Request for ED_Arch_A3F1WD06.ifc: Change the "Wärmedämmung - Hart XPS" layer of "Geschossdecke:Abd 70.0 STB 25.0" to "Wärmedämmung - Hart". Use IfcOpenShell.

First a look at what the model holds.

```python
import ifcopenshell
import ifcopenshell.util.element

model = ifcopenshell.open("ED_Arch_A3F1WD06.ifc")
print(model.schema)
for layer_set in model.by_type("IfcMaterialLayerSet"):
    if layer_set.LayerSetName == "Geschossdecke:Abd 70.0 STB 25.0":
        for layer in layer_set.MaterialLayers:
            print(layer.id(), layer.Material and layer.Material.Name, layer.LayerThickness, sep=" | ")
        print(len(ifcopenshell.util.element.get_elements_by_material(model, layer_set)), "elements and types use it")
print(sorted(m.Name for m in model.by_type("IfcMaterial") if m.Name)[:60])
```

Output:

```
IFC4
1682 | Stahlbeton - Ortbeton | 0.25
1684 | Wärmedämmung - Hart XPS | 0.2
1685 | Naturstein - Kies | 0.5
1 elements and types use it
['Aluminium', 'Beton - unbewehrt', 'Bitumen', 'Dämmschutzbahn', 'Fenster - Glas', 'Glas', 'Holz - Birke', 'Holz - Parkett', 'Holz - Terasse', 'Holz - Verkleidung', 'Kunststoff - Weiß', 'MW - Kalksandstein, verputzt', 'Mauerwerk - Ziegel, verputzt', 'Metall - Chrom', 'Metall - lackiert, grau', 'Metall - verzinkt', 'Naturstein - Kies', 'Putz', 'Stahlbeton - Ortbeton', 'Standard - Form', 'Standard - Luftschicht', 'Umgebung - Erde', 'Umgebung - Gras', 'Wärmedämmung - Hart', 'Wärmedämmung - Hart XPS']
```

```python
import ifcopenshell
import ifcopenshell.api.material

model = ifcopenshell.open("ED_Arch_A3F1WD06.ifc")

layer_set = next(s for s in model.by_type("IfcMaterialLayerSet") if s.LayerSetName == "Geschossdecke:Abd 70.0 STB 25.0")
layer = next(l for l in layer_set.MaterialLayers if l.Material and l.Material.Name == "Wärmedämmung - Hart XPS")
material = next(m for m in model.by_type("IfcMaterial") if m.Name == "Wärmedämmung - Hart")

# Point this one layer at the other material; renaming the old one would change it everywhere.
ifcopenshell.api.material.edit_layer(model, layer=layer, attributes={}, material=material)

print([l.Material.Name if l.Material else None for l in layer_set.MaterialLayers])

model.write("ED_Arch_A3F1WD06_v2.ifc")
```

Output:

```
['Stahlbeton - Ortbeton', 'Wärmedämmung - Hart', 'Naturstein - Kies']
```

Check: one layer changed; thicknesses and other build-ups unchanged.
